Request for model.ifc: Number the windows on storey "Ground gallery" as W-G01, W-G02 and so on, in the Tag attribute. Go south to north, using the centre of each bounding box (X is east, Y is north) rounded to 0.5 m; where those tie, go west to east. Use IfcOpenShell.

First a look at what the model holds.

```python
import ifcopenshell
import ifcopenshell.util.element
import ifcopenshell.util.placement

model = ifcopenshell.open("model.ifc")
print(model.schema)
storey = next(s for s in model.by_type("IfcBuildingStorey") if s.Name == "Ground gallery")
windows = [e for e in ifcopenshell.util.element.get_decomposition(storey) if e.is_a("IfcWindow")]
for e in sorted(windows, key=lambda e: e.id()):
    origin = ifcopenshell.util.placement.get_local_placement(e.ObjectPlacement)[:3, 3]
    print(e.id(), e.Tag, e.Name, origin.round(2) + 0.0, sep=" | ")
```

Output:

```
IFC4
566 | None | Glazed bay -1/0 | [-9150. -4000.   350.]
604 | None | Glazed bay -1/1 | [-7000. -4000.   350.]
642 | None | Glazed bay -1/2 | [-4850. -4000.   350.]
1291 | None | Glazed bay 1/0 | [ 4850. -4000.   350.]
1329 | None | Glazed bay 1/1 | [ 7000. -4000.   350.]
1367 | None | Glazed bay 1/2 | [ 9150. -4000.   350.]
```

```python
import ifcopenshell
import ifcopenshell.geom
import ifcopenshell.util.element
import ifcopenshell.util.shape

model = ifcopenshell.open("model.ifc")
settings = ifcopenshell.geom.settings()
settings.set("use-world-coords", True)


def centre(element):
    shape = ifcopenshell.geom.create_shape(settings, element)
    return ifcopenshell.util.shape.get_bbox_centroid(shape.geometry)


storey = next(s for s in model.by_type("IfcBuildingStorey") if s.Name == "Ground gallery")
windows = [e for e in ifcopenshell.util.element.get_decomposition(storey) if e.is_a("IfcWindow")]

# Insertion points can sit at a corner or the storey origin, so sort by the geometry (in metres).
centres = {e: centre(e) for e in windows}
windows.sort(key=lambda e: (round(centres[e][1] / 0.5), centres[e][0]))

for i, e in enumerate(windows, start=1):
    number = f"W-G{i:02d}"
    e.Tag = number
    print(e.id(), number)

model.write("model_updated.ifc")
```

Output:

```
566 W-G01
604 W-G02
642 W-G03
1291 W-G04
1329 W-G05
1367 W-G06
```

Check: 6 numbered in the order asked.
